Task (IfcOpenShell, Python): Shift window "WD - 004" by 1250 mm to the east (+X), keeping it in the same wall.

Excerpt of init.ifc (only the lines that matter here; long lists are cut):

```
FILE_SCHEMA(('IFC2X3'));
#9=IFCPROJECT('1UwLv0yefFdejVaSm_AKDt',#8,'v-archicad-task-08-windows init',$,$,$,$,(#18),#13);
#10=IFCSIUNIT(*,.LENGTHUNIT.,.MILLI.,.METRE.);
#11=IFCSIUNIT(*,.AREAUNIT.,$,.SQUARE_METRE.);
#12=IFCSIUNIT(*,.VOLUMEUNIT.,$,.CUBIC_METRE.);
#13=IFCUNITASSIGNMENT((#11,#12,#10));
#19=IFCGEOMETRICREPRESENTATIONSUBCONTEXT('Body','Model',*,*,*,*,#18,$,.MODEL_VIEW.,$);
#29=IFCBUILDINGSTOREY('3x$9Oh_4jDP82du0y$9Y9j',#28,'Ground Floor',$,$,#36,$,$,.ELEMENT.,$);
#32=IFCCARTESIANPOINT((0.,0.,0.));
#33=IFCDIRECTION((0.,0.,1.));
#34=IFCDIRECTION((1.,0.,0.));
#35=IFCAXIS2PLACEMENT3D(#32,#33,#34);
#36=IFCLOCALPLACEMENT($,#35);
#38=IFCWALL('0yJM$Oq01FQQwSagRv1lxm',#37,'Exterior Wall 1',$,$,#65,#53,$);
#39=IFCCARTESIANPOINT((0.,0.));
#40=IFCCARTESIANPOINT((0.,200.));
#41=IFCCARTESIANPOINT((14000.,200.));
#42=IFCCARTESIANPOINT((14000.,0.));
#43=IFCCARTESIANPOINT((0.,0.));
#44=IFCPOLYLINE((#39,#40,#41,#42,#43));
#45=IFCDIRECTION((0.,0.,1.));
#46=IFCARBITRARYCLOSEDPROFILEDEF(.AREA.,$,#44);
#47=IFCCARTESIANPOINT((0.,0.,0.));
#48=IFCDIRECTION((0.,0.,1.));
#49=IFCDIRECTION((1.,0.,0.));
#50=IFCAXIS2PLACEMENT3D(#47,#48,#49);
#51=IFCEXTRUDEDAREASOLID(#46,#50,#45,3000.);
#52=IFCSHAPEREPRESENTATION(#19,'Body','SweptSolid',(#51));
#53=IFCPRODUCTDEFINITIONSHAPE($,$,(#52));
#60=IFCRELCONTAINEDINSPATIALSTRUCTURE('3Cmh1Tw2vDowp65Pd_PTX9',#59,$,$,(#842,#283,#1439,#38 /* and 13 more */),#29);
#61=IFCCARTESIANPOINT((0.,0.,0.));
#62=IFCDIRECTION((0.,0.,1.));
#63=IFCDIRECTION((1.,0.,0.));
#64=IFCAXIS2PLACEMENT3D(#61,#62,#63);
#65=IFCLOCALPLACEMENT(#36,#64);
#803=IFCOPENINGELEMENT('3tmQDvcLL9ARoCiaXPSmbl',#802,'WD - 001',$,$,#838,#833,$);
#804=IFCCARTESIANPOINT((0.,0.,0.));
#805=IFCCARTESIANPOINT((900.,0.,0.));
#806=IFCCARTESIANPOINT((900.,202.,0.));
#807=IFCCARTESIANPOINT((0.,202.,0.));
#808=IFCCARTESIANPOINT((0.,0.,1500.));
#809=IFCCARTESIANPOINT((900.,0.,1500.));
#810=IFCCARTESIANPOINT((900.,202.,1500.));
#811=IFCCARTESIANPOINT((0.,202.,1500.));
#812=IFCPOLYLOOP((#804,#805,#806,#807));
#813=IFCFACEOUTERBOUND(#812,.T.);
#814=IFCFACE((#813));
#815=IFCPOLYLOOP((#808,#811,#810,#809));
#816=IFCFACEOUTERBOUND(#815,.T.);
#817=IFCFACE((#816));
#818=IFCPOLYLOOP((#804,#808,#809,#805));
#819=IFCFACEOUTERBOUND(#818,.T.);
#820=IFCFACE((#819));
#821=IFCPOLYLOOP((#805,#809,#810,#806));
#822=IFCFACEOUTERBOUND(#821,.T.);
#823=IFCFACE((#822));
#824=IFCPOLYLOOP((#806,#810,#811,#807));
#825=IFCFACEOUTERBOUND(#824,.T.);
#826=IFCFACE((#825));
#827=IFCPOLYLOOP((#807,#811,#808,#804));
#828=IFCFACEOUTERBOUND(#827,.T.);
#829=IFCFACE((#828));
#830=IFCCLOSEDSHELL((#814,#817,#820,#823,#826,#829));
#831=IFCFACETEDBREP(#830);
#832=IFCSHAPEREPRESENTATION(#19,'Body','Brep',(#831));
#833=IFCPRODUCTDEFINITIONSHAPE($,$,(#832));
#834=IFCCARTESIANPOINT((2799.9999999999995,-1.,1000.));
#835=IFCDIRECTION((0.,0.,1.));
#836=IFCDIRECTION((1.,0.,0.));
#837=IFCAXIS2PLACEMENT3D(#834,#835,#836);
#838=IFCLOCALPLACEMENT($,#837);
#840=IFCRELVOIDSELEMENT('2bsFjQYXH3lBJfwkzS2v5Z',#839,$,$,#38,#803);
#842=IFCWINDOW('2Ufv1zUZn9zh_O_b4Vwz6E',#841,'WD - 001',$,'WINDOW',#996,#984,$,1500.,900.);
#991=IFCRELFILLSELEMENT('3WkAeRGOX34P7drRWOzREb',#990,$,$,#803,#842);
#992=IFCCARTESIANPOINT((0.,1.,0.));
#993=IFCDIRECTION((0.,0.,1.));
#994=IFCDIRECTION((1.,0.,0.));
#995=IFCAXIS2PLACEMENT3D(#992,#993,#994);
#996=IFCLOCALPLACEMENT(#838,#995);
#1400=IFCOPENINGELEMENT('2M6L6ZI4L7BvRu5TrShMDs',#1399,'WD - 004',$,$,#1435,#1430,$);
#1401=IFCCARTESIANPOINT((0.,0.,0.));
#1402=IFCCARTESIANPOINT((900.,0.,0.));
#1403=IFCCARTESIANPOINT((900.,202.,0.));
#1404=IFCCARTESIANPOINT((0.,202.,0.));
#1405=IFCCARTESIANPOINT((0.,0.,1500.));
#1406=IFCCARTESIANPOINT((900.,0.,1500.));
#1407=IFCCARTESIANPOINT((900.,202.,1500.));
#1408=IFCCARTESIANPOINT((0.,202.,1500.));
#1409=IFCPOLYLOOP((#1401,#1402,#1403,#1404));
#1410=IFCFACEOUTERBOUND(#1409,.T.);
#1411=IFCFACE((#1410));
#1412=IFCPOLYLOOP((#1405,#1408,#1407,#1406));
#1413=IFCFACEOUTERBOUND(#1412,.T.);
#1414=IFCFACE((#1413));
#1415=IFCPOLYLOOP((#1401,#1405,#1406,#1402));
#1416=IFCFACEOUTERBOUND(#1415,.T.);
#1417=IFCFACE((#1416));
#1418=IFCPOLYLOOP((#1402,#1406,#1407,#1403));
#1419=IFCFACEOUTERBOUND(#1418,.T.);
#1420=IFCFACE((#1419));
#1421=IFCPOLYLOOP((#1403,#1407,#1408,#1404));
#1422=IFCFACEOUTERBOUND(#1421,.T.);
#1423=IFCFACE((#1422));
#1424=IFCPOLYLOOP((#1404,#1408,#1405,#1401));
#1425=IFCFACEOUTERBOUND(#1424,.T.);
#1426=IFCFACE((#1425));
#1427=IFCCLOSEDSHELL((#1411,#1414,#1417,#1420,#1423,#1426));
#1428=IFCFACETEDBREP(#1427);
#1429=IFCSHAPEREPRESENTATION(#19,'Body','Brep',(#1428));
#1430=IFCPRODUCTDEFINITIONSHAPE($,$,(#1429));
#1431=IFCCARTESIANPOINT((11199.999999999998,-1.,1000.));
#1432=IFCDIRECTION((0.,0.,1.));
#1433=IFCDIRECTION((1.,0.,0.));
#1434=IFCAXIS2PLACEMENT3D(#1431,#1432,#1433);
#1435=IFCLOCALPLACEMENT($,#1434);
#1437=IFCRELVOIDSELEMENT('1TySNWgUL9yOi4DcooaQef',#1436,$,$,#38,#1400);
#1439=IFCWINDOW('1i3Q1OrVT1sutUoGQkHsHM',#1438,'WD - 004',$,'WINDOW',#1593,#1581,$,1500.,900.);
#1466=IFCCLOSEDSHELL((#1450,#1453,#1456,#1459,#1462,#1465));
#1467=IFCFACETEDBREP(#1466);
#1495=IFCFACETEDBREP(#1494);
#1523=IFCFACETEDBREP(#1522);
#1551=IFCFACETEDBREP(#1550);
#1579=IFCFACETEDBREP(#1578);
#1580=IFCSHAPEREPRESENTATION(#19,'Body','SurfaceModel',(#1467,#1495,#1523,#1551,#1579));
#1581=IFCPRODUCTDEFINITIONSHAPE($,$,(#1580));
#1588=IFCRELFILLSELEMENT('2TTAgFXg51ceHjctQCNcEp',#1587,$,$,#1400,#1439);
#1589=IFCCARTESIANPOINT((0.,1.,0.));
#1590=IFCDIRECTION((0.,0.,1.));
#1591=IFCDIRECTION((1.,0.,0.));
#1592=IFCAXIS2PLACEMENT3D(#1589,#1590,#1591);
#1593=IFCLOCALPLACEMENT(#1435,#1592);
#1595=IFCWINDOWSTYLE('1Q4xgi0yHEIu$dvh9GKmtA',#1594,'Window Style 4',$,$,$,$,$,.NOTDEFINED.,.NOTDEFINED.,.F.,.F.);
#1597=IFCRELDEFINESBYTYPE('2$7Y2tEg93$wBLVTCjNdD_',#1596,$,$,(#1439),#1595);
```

```python
import ifcopenshell
import ifcopenshell.api.geometry
import ifcopenshell.util.placement
import ifcopenshell.util.unit

model = ifcopenshell.open("init.ifc")
unit_scale = ifcopenshell.util.unit.calculate_unit_scale(model)

window = model.by_id(1439)
opening = window.FillsVoids[0].RelatingOpeningElement
wall = opening.VoidsElements[0].RelatingBuildingElement

wall_matrix = ifcopenshell.util.placement.get_local_placement(wall.ObjectPlacement)
shift = wall_matrix[:3, 0] * 1.25 / unit_scale
before = ifcopenshell.util.placement.get_local_placement(window.ObjectPlacement)[:3, 3].copy()

# The window is placed relative to its opening, so it follows when the opening moves.
matrix = ifcopenshell.util.placement.get_local_placement(opening.ObjectPlacement)
matrix[:3, 3] += shift
ifcopenshell.api.geometry.edit_object_placement(
    model, product=opening, matrix=matrix, is_si=False, should_transform_children=True
)

after = ifcopenshell.util.placement.get_local_placement(window.ObjectPlacement)[:3, 3]
print("window moved by", (after - before).round(3) + 0.0)

model.write("init_edited.ifc")
```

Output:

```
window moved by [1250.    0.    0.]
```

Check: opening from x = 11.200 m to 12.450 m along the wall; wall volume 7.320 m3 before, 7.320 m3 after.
